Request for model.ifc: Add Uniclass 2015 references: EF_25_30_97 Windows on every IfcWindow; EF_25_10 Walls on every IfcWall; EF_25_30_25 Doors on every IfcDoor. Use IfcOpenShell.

First a look at what the model holds.

```python
import ifcopenshell

model = ifcopenshell.open("model.ifc")
print(model.schema)
print("classifications:", [c.Name for c in model.by_type("IfcClassification")])
for ifc_class in ("IfcDoor", "IfcRoof", "IfcStair", "IfcWall", "IfcWindow"):
    print(ifc_class, len(model.by_type(ifc_class)))
```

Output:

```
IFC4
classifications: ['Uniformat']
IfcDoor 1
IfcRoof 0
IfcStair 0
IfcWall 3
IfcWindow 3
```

```python
import ifcopenshell
import ifcopenshell.api.classification

model = ifcopenshell.open("model.ifc")

system = ifcopenshell.api.classification.add_classification(model, classification="Uniclass 2015")

codes = {
    "IfcWindow": ("EF_25_30_97", "Windows"),
    "IfcWall": ("EF_25_10", "Walls"),
    "IfcDoor": ("EF_25_30_25", "Doors"),
}
for ifc_class, (code, name) in codes.items():
    products = model.by_type(ifc_class)
    ifcopenshell.api.classification.add_reference(
        model, products=products, classification=system, identification=code, name=name
    )
    print(code, len(products))

model.write("model_edited.ifc")
```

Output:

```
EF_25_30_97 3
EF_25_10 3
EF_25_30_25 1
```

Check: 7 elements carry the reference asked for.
